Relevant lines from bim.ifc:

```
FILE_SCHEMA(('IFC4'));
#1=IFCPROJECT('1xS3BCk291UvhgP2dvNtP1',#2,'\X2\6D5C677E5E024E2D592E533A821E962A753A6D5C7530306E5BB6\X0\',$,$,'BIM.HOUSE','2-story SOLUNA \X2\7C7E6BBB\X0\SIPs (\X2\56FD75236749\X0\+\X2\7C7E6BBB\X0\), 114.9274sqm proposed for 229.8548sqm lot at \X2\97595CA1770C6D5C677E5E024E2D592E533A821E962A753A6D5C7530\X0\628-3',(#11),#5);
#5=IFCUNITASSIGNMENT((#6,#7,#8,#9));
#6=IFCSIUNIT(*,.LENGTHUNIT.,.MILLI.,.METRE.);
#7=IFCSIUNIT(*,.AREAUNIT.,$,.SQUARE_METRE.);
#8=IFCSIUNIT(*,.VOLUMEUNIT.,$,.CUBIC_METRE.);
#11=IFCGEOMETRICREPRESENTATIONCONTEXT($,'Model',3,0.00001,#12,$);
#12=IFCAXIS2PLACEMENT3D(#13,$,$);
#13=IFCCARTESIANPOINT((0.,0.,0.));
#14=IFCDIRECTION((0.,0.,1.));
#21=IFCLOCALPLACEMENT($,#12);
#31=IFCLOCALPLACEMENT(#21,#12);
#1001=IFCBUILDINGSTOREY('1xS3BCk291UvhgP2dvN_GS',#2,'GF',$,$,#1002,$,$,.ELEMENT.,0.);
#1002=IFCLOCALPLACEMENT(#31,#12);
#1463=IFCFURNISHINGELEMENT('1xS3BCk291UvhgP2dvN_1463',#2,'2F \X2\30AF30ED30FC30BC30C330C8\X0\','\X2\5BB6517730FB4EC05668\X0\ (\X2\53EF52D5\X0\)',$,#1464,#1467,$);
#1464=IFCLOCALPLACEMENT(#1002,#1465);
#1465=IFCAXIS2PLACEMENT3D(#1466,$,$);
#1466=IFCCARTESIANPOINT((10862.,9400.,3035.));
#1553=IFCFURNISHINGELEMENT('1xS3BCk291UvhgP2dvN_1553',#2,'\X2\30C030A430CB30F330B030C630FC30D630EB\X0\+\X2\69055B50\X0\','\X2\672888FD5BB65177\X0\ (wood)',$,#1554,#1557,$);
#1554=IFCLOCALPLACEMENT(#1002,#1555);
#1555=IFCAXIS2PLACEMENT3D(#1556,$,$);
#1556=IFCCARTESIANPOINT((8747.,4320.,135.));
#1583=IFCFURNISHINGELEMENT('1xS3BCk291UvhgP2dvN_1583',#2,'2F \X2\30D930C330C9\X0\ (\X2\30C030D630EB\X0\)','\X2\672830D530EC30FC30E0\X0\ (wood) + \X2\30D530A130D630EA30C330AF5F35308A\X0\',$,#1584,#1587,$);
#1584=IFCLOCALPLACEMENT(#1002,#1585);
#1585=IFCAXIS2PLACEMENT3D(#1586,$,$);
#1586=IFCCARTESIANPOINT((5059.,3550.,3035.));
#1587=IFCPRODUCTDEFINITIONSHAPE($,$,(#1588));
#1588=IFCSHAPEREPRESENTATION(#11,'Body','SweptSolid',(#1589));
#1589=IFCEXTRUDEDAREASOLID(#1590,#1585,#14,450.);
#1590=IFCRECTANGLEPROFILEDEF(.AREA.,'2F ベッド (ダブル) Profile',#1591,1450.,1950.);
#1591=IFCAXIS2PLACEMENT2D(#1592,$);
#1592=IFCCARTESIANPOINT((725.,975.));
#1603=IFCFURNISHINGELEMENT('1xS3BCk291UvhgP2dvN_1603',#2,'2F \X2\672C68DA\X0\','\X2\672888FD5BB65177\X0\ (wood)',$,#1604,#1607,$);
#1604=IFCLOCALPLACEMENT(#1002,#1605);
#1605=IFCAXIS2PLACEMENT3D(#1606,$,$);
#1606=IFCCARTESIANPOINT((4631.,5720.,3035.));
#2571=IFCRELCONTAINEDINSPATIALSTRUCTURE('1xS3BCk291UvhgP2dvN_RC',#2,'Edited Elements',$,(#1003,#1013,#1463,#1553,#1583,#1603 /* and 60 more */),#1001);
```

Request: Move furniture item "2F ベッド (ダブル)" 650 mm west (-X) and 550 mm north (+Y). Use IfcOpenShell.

```python
import ifcopenshell
import ifcopenshell.api.geometry
import ifcopenshell.util.placement
import ifcopenshell.util.unit

model = ifcopenshell.open("bim.ifc")
unit_scale = ifcopenshell.util.unit.calculate_unit_scale(model)

item = model.by_guid("1xS3BCk291UvhgP2dvN_1583")
matrix = ifcopenshell.util.placement.get_local_placement(item.ObjectPlacement)
matrix[0, 3] -= 0.65 / unit_scale
matrix[1, 3] += 0.55 / unit_scale
ifcopenshell.api.geometry.edit_object_placement(model, product=item, matrix=matrix, is_si=False)

print(ifcopenshell.util.placement.get_local_placement(item.ObjectPlacement).round(3) + 0.0)

model.write("bim_rev.ifc")
```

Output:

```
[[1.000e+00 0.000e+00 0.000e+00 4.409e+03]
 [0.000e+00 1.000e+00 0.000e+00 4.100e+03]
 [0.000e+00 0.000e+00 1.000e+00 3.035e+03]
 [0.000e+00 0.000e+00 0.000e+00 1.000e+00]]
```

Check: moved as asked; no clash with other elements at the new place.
